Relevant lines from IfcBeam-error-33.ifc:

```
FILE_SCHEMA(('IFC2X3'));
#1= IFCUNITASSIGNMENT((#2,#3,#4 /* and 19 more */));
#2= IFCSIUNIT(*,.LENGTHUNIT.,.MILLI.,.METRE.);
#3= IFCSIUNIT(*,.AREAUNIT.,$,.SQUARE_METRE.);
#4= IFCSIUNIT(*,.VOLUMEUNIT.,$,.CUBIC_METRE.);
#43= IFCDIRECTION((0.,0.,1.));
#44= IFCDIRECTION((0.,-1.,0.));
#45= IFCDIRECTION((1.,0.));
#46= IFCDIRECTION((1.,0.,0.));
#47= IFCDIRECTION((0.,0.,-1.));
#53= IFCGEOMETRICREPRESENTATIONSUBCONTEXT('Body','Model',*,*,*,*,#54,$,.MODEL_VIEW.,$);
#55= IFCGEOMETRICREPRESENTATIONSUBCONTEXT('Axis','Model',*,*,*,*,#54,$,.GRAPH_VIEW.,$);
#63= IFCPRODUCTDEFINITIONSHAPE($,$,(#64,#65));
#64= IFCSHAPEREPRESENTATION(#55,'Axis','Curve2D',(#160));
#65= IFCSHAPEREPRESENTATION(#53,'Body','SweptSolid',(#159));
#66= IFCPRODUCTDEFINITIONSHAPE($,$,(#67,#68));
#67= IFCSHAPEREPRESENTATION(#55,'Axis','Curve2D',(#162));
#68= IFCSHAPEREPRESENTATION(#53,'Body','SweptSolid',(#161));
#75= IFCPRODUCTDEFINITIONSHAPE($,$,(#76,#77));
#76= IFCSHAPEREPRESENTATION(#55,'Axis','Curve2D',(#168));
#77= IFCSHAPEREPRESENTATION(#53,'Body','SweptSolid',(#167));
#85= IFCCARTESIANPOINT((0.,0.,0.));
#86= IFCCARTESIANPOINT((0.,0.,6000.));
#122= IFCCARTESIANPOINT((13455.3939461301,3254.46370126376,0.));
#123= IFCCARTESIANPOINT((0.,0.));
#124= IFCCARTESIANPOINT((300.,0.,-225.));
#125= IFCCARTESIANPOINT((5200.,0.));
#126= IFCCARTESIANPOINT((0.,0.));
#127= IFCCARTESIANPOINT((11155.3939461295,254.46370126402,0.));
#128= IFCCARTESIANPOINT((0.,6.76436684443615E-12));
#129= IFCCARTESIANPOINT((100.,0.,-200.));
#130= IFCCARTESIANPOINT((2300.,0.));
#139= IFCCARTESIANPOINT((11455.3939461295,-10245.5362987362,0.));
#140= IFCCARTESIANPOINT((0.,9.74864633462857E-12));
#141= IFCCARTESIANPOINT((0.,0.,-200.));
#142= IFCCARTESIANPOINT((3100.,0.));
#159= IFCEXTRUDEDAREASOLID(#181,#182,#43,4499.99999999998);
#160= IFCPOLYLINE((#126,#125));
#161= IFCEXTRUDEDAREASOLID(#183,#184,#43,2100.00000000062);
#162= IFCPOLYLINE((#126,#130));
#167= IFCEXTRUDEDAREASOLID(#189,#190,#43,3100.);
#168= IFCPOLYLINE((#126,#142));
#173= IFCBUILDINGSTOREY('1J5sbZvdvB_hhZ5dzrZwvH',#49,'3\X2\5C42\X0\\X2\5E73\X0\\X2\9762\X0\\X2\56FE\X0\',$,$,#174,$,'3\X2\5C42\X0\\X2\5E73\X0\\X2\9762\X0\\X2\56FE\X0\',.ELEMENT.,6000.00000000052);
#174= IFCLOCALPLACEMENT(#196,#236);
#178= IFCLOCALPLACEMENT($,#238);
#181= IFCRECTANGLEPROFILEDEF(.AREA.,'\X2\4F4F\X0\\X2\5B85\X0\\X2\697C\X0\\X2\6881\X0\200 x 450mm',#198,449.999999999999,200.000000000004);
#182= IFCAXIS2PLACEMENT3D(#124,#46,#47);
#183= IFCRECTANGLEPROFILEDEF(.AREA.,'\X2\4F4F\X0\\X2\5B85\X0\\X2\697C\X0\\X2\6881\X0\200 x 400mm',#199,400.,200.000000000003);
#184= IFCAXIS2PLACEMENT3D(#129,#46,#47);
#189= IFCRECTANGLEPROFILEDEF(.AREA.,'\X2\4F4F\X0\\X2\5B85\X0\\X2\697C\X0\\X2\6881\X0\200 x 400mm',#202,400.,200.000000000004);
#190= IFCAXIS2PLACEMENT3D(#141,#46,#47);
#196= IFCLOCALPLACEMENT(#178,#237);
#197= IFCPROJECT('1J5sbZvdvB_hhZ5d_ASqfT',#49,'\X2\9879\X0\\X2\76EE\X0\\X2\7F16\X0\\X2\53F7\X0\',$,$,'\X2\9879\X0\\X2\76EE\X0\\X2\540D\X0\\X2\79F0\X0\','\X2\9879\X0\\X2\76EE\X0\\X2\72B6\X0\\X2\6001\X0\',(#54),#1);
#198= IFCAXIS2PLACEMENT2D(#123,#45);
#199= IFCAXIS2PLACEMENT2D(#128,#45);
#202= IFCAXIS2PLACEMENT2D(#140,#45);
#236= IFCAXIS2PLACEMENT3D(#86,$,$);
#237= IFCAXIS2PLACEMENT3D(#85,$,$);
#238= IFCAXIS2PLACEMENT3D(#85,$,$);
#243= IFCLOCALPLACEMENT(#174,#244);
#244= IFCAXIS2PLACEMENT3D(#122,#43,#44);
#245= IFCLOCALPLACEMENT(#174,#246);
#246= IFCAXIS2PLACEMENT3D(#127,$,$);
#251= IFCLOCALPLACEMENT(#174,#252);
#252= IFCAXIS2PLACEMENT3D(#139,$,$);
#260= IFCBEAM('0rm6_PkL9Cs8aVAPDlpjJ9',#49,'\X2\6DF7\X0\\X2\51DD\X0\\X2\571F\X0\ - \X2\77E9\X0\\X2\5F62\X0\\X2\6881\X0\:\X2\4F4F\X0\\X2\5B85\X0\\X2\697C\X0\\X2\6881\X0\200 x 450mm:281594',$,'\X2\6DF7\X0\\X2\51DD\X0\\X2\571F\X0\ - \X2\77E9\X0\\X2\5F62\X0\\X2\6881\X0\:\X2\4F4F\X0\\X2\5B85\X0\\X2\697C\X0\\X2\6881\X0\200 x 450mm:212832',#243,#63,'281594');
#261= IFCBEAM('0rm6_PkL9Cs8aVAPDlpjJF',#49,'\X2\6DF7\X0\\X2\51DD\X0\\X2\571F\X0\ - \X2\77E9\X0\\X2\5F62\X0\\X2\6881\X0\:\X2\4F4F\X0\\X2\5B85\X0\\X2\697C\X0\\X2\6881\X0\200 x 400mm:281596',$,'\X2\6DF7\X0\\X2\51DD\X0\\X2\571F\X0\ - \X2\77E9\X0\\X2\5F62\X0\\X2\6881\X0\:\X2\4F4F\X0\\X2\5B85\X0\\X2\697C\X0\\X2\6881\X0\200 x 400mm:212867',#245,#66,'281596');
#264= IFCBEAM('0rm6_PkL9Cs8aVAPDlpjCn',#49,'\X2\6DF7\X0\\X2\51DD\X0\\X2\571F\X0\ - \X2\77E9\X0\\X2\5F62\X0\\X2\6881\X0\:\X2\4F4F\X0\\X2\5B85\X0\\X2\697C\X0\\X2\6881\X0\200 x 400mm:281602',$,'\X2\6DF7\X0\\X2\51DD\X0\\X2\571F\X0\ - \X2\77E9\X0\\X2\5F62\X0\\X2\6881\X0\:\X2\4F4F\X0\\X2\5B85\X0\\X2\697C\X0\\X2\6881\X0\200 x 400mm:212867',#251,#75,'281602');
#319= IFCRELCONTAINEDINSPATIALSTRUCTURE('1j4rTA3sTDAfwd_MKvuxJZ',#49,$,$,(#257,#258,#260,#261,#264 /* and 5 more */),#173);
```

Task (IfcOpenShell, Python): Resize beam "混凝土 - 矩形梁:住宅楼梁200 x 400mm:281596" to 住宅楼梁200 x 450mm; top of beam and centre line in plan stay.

```python
import ifcopenshell
import ifcopenshell.util.element
import ifcopenshell.util.representation

model = ifcopenshell.open("IfcBeam-error-33.ifc")

member = model.by_guid("0rm6_PkL9Cs8aVAPDlpjJF")
source = next(p for p in model.by_type("IfcRectangleProfileDef") if p.ProfileName == "住宅楼梁200 x 450mm")

body = ifcopenshell.util.representation.get_representation(member, "Model", "Body")
solid = body.Items[0]
old_profile = solid.SweptArea

# Copy the section's sizes but keep this member's own profile position.
profile = ifcopenshell.util.element.copy(model, source)
# Profiles are centred, so shift by half the change in depth to hold the top.
shift = (old_profile.XDim - profile.XDim) / 2
x, y = old_profile.Position.Location.Coordinates
up = (-1.0, 0.0)  # upwards, in the solid's own plane
location = model.createIfcCartesianPoint((x + up[0] * shift, y + up[1] * shift))
profile.Position = model.createIfcAxis2Placement2D(location, old_profile.Position.RefDirection)
solid.SweptArea = profile
if not model.get_total_inverses(old_profile):
    ifcopenshell.util.element.remove_deep2(model, old_profile)
member.Name = member.Name.replace("住宅楼梁200 x 400mm", "住宅楼梁200 x 450mm")
member.ObjectType = member.ObjectType.replace("住宅楼梁200 x 400mm", "住宅楼梁200 x 450mm")

print(solid.SweptArea)

model.write("IfcBeam-error-33_rev.ifc")
```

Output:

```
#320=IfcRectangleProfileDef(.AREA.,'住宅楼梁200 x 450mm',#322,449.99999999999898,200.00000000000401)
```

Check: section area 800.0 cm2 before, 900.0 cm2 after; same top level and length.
